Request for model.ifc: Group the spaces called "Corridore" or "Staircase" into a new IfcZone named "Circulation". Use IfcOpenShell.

First a look at what the model holds.

```python
import ifcopenshell

model = ifcopenshell.open("model.ifc")
print(model.schema)
seen = {}
for space in model.by_type("IfcSpace"):
    seen[space.LongName] = seen.get(space.LongName, 0) + 1
for name, count in sorted(seen.items(), key=str):
    print(count, "x", name)
print("zones:", [z.Name for z in model.by_type("IfcZone")][:20])
```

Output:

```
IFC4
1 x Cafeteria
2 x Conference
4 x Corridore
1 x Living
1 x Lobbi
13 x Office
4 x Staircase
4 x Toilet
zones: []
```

```python
import ifcopenshell
import ifcopenshell.api.group
import ifcopenshell.api.root

model = ifcopenshell.open("model.ifc")

names = {"Corridore", "Staircase"}
spaces = [s for s in model.by_type("IfcSpace") if s.LongName in names]

zone = ifcopenshell.api.root.create_entity(model, ifc_class="IfcZone", name="Circulation")
ifcopenshell.api.group.assign_group(model, products=spaces, group=zone)
print(len(spaces), "spaces in", zone.Name)

model.write("model_edited.ifc")
```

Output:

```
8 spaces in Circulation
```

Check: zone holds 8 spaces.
